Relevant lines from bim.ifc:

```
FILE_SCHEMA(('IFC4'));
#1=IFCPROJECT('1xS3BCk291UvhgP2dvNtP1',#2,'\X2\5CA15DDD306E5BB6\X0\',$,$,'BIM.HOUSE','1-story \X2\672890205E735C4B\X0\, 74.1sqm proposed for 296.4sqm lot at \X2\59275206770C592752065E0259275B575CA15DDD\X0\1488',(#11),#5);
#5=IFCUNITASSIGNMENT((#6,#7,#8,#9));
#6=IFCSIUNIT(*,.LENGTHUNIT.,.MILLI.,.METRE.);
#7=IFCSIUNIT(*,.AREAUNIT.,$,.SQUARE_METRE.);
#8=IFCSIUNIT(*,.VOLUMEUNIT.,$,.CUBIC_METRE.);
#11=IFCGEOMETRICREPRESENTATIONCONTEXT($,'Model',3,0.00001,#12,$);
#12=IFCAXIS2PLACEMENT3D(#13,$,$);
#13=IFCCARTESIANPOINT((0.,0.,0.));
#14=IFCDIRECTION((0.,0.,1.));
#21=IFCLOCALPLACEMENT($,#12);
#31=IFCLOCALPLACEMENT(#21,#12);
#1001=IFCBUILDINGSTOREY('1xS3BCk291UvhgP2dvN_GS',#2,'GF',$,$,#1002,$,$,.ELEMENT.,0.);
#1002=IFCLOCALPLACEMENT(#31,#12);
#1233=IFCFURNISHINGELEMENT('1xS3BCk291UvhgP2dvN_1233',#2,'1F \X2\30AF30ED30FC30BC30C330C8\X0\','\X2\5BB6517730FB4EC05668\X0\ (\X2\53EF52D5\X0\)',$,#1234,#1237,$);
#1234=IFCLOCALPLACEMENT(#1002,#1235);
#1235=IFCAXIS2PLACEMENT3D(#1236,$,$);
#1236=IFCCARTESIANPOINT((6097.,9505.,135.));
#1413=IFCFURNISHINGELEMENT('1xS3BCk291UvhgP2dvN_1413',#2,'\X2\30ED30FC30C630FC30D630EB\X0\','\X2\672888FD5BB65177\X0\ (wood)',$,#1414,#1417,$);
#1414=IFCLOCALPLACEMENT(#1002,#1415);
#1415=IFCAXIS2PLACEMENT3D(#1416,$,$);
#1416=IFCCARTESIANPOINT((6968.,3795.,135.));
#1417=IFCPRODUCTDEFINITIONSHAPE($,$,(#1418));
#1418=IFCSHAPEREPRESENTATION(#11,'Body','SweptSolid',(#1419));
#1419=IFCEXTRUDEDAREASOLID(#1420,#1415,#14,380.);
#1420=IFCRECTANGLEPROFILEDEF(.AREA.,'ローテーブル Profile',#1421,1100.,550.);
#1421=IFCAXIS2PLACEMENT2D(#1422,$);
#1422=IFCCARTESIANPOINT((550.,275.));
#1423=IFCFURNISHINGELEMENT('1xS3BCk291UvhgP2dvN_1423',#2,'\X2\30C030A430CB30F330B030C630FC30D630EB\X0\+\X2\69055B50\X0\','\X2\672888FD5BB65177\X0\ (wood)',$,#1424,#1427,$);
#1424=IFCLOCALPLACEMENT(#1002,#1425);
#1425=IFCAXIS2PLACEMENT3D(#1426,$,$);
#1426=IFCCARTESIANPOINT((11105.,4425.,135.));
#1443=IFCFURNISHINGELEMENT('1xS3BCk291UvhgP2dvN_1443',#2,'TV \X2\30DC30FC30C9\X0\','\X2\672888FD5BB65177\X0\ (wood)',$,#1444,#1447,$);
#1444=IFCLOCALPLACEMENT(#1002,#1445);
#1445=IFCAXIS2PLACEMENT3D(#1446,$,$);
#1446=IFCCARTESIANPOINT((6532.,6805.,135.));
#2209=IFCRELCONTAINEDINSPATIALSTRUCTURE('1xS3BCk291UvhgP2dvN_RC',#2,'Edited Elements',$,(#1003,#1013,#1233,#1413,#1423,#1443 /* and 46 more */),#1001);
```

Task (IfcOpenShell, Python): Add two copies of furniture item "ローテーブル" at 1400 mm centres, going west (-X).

```python
import numpy as np
import ifcopenshell
import ifcopenshell.api.geometry
import ifcopenshell.api.root
import ifcopenshell.util.element
import ifcopenshell.util.placement

model = ifcopenshell.open("bim.ifc")


def reuse_history(source, copy):
    """copy_class also copies each property set's owner history, people and application; keep the originals."""
    for rel in copy.IsDefinedBy:
        if rel.is_a("IfcRelDefinesByProperties") and (history := rel.RelatingPropertyDefinition.OwnerHistory):
            rel.RelatingPropertyDefinition.OwnerHistory = source.OwnerHistory
            ifcopenshell.util.element.remove_deep2(model, history)


source = model.by_guid("1xS3BCk291UvhgP2dvN_1413")
base = ifcopenshell.util.placement.get_local_placement(source.ObjectPlacement)
step = np.array([-1.0, 0.0, 0.0]) * 1400.0

for i in range(1, 3):
    copy = ifcopenshell.api.root.copy_class(model, product=source)
    copy.Representation = ifcopenshell.util.element.copy_deep(
        model, source.Representation, exclude=["IfcGeometricRepresentationContext", "IfcRepresentationMap"]
    )
    reuse_history(source, copy)
    matrix = base.copy()
    matrix[:3, 3] += i * step
    print("added at", matrix[:3, 3].round(3) + 0.0)
    ifcopenshell.api.geometry.edit_object_placement(model, product=copy, matrix=matrix, is_si=False)

model.write("bim_rev.ifc")
```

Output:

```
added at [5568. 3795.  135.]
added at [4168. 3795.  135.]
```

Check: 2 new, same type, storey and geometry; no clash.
